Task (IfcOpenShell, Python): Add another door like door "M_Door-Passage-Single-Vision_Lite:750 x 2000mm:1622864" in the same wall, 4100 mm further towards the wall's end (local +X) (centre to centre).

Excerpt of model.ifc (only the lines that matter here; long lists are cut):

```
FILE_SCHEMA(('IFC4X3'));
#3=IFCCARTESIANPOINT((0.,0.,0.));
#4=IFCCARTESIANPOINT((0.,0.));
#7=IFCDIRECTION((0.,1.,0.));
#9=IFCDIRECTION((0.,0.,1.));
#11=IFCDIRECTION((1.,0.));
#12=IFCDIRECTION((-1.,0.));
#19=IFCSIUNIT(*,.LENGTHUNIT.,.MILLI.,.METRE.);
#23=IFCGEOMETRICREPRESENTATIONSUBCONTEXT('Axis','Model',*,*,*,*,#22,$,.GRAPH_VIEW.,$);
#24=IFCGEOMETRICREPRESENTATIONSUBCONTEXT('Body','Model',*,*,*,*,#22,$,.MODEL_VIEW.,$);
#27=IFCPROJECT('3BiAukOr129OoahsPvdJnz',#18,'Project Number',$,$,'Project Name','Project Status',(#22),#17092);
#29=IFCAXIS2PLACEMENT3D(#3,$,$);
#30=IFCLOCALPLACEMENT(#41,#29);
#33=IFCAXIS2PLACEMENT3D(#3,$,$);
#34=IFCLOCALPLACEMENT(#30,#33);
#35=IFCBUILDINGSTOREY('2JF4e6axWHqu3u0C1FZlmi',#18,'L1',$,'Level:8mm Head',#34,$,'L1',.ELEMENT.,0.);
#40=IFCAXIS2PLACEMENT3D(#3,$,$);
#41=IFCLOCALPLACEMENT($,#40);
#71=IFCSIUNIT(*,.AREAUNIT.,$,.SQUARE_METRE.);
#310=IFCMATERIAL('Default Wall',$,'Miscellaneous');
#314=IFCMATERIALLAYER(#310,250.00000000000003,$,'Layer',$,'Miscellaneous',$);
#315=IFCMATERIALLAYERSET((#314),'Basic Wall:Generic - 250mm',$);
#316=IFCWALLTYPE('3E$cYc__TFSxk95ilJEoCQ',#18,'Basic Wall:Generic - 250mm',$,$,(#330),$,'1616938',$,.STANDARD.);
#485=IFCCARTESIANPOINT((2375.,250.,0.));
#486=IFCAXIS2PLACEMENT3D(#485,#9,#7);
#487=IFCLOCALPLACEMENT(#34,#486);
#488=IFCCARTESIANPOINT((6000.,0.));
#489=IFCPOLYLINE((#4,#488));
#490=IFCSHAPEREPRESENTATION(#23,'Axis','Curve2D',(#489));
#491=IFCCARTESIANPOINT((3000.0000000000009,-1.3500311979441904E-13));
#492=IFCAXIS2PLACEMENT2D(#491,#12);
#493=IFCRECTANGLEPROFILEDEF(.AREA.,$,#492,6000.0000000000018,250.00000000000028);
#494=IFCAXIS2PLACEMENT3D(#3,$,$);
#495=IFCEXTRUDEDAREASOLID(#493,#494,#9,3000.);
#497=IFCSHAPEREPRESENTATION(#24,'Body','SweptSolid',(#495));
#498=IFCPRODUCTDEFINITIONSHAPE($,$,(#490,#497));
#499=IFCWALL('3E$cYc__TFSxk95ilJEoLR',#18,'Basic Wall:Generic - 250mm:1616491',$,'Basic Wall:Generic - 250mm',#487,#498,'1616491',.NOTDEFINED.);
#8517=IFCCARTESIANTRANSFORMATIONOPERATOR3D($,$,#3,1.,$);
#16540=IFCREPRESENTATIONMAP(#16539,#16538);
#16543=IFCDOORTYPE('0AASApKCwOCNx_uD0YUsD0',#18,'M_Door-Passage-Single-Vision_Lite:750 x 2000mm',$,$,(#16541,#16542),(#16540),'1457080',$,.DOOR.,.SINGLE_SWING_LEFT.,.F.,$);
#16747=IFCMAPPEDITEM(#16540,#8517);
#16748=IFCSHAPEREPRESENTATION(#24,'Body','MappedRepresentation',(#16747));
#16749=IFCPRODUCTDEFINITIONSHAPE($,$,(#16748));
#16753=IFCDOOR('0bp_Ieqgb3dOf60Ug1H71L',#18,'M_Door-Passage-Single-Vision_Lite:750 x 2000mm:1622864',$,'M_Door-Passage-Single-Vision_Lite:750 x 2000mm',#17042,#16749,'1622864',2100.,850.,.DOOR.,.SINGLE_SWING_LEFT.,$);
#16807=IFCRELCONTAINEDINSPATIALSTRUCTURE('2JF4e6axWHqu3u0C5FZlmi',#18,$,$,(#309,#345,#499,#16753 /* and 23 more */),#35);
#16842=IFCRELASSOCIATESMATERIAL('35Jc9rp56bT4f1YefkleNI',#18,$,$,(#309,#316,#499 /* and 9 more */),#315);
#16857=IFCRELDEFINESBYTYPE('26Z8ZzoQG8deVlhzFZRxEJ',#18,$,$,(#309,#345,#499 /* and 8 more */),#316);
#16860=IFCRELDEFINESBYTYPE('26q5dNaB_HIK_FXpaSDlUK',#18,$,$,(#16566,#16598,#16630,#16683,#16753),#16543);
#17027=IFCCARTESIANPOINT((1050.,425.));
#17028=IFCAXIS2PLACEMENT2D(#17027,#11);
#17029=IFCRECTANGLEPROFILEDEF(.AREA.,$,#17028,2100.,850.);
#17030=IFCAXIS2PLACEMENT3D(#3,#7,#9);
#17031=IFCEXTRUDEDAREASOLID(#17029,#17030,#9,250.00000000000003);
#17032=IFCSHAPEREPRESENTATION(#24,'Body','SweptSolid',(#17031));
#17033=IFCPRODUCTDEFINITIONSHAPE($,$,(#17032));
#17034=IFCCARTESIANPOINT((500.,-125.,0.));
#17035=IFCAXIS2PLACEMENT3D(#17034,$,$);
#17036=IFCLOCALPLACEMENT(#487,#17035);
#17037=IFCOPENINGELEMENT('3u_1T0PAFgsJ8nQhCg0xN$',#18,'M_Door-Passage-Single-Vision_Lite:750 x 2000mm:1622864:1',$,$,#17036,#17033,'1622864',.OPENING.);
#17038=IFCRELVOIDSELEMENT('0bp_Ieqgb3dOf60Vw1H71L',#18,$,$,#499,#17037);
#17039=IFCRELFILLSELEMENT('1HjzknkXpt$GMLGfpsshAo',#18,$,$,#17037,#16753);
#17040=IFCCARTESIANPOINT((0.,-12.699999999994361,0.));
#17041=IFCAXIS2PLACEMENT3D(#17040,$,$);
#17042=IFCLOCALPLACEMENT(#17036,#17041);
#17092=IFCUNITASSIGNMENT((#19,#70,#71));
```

```python
import ifcopenshell
import ifcopenshell.api.feature
import ifcopenshell.api.geometry
import ifcopenshell.api.root
import ifcopenshell.geom
import ifcopenshell.util.element
import ifcopenshell.util.placement
import ifcopenshell.util.shape

model = ifcopenshell.open("model.ifc")
settings = ifcopenshell.geom.settings()


def volume(element):
    """Net volume in cubic metres, openings subtracted."""
    shape = ifcopenshell.geom.create_shape(settings, element)
    return ifcopenshell.util.shape.get_volume(shape.geometry)


def reuse_history(source, copy):
    """copy_class also copies each property set's owner history, people and application; keep the originals."""
    for rel in copy.IsDefinedBy:
        if rel.is_a("IfcRelDefinesByProperties") and (history := rel.RelatingPropertyDefinition.OwnerHistory):
            rel.RelatingPropertyDefinition.OwnerHistory = source.OwnerHistory
            ifcopenshell.util.element.remove_deep2(model, history)


door = model.by_guid("0bp_Ieqgb3dOf60Ug1H71L")
opening = door.FillsVoids[0].RelatingOpeningElement
wall = opening.VoidsElements[0].RelatingBuildingElement
before = volume(wall)
shift = ifcopenshell.util.placement.get_local_placement(wall.ObjectPlacement)[:3, 0] * 4100.0

# copy_class copies the void relationship, type, container and properties, but no geometry.
new_opening = ifcopenshell.api.root.copy_class(model, product=opening)
new_opening.Representation = ifcopenshell.util.element.copy_deep(
    model, opening.Representation, exclude=["IfcGeometricRepresentationContext", "IfcRepresentationMap"]
)
new_opening.Name = "M_Door-Passage-Single-Vision_Lite:750 x 2000mm"
new_opening.Tag = None
new_door = ifcopenshell.api.root.copy_class(model, product=door)
new_door.Representation = ifcopenshell.util.element.copy_deep(
    model, door.Representation, exclude=["IfcGeometricRepresentationContext", "IfcRepresentationMap"]
)
new_door.Name = "M_Door-Passage-Single-Vision_Lite:750 x 2000mm"
new_door.Tag = None
reuse_history(door, new_door)
ifcopenshell.api.feature.add_filling(model, opening=new_opening, element=new_door)

for old, new in ((opening, new_opening), (door, new_door)):
    matrix = ifcopenshell.util.placement.get_local_placement(old.ObjectPlacement)
    matrix[:3, 3] += shift
    ifcopenshell.api.geometry.edit_object_placement(model, product=new, matrix=matrix, is_si=False)

after = volume(wall)

print(f"wall volume {before:.3f} -> {after:.3f} m3")

model.write("model-out.ifc")
```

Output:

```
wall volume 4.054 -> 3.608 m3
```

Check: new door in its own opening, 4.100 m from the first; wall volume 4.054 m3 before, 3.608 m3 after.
